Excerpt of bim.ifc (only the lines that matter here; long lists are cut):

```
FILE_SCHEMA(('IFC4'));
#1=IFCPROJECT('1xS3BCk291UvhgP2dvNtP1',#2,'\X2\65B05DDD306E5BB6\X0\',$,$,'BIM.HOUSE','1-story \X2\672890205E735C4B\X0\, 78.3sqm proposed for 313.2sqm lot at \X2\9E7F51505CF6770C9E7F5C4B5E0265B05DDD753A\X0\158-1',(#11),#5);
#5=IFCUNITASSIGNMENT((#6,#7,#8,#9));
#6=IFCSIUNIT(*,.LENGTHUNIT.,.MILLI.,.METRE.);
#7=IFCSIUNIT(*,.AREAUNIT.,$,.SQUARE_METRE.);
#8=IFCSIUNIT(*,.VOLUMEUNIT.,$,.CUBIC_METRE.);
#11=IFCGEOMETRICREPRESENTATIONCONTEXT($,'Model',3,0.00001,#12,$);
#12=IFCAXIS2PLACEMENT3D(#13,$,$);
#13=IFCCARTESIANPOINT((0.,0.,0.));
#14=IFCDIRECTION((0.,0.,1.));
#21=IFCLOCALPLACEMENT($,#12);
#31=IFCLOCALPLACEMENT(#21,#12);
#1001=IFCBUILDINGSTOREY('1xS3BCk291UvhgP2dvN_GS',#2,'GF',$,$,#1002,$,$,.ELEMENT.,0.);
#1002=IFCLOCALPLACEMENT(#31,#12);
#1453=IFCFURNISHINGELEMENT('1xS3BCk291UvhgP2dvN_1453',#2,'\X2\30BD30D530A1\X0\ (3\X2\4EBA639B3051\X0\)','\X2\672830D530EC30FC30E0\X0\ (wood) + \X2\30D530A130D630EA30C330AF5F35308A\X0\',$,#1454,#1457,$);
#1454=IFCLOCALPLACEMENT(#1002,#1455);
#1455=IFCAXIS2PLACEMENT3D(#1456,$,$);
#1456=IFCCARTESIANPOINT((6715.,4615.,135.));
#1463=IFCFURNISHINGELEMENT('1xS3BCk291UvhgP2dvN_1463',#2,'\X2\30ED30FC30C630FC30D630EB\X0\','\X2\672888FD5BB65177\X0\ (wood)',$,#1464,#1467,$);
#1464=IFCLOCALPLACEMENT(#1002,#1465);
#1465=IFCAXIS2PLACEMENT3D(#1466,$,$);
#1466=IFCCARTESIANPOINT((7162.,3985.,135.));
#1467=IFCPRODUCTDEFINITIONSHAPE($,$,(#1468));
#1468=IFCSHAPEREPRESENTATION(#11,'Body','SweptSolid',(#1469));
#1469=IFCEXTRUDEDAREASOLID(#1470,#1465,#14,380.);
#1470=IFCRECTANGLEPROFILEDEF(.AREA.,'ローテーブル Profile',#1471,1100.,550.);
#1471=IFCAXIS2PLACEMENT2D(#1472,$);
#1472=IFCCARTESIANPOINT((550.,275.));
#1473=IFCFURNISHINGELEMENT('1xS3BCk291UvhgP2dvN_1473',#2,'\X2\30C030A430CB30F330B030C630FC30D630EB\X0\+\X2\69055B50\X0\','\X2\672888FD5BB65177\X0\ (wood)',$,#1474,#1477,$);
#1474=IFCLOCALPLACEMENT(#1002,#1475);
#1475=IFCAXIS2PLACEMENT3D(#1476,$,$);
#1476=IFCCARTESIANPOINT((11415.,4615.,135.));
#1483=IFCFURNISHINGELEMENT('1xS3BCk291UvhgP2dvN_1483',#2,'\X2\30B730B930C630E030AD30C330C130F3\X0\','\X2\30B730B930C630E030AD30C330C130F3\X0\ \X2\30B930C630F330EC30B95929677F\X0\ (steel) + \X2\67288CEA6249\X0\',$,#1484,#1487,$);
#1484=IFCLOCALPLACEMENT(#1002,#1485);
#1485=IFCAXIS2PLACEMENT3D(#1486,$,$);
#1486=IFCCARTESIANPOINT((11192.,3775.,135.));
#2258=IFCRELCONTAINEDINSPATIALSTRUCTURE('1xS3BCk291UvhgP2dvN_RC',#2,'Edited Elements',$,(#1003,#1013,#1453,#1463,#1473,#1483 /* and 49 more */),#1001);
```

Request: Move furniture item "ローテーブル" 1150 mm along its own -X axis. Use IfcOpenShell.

```python
import ifcopenshell
import ifcopenshell.api.geometry
import ifcopenshell.util.placement
import ifcopenshell.util.unit

model = ifcopenshell.open("bim.ifc")
unit_scale = ifcopenshell.util.unit.calculate_unit_scale(model)

item = model.by_guid("1xS3BCk291UvhgP2dvN_1463")
matrix = ifcopenshell.util.placement.get_local_placement(item.ObjectPlacement)
matrix[:3, 3] -= matrix[:3, 0] * 1.15 / unit_scale
ifcopenshell.api.geometry.edit_object_placement(model, product=item, matrix=matrix, is_si=False)

print(ifcopenshell.util.placement.get_local_placement(item.ObjectPlacement).round(3) + 0.0)

model.write("bim-out.ifc")
```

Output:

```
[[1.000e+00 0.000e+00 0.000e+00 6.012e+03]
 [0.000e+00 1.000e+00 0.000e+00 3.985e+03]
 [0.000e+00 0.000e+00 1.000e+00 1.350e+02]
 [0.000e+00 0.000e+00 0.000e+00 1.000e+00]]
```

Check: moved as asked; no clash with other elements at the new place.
